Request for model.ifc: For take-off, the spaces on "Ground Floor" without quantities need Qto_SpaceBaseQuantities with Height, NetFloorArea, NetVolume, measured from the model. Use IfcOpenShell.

First a look at what the model holds.

```python
import ifcopenshell
import ifcopenshell.util.element
import ifcopenshell.util.unit

model = ifcopenshell.open("model.ifc")
print(model.schema)
for unit_type in ("LENGTHUNIT", "AREAUNIT", "VOLUMEUNIT"):
    print(unit_type, ifcopenshell.util.unit.calculate_unit_scale(model, unit_type))
storey = next(s for s in model.by_type("IfcBuildingStorey") if s.Name == "Ground Floor")
spaces = [e for e in ifcopenshell.util.element.get_decomposition(storey) if e.is_a("IfcSpace")]
for e in sorted(spaces, key=lambda e: e.id()):
    print(e.id(), e.is_a(), e.Name, list(ifcopenshell.util.element.get_psets(e, qtos_only=True)), sep=" | ")
```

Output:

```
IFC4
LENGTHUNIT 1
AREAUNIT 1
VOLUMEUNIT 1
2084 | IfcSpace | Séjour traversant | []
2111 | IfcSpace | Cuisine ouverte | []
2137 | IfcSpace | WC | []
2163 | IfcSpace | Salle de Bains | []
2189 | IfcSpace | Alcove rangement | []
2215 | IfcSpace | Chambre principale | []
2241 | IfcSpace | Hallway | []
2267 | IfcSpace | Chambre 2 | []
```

```python
import ifcopenshell
import ifcopenshell.api.pset
import ifcopenshell.geom
import ifcopenshell.util.element
import ifcopenshell.util.shape
import ifcopenshell.util.unit

model = ifcopenshell.open("model.ifc")
unit_scale = ifcopenshell.util.unit.calculate_unit_scale(model)
area_scale = ifcopenshell.util.unit.calculate_unit_scale(model, "AREAUNIT")
volume_scale = ifcopenshell.util.unit.calculate_unit_scale(model, "VOLUMEUNIT")
settings = ifcopenshell.geom.settings()

storey = next(s for s in model.by_type("IfcBuildingStorey") if s.Name == "Ground Floor")
spaces = [e for e in ifcopenshell.util.element.get_decomposition(storey) if e.is_a("IfcSpace")]

for e in sorted(spaces, key=lambda e: e.id()):
    if ifcopenshell.util.element.get_psets(e, qtos_only=True, should_inherit=False):
        continue
    # Geometry comes back in metres, in the element's own axes.
    shape = ifcopenshell.geom.create_shape(settings, e)
    values = {
        "Height": ifcopenshell.util.shape.get_z(shape.geometry) / unit_scale,
        "NetFloorArea": ifcopenshell.util.shape.get_footprint_area(shape.geometry) / area_scale,
        "NetVolume": ifcopenshell.util.shape.get_volume(shape.geometry) / volume_scale,
    }
    qto = ifcopenshell.api.pset.add_qto(model, product=e, name="Qto_SpaceBaseQuantities")
    ifcopenshell.api.pset.edit_qto(model, qto=qto, properties=values)
    print(e.id(), {k: round(v, 3) for k, v in values.items()})

model.write("model_rev.ifc")
```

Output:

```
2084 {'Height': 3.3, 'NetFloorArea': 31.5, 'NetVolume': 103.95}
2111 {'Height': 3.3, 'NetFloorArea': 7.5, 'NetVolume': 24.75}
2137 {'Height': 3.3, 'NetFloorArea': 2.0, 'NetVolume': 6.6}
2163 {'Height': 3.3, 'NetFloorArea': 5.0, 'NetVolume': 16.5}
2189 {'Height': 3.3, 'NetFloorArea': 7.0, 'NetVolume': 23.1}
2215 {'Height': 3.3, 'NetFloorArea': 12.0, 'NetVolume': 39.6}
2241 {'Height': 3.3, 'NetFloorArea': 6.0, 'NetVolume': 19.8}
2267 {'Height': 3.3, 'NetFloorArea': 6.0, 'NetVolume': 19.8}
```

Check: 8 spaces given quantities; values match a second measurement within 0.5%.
